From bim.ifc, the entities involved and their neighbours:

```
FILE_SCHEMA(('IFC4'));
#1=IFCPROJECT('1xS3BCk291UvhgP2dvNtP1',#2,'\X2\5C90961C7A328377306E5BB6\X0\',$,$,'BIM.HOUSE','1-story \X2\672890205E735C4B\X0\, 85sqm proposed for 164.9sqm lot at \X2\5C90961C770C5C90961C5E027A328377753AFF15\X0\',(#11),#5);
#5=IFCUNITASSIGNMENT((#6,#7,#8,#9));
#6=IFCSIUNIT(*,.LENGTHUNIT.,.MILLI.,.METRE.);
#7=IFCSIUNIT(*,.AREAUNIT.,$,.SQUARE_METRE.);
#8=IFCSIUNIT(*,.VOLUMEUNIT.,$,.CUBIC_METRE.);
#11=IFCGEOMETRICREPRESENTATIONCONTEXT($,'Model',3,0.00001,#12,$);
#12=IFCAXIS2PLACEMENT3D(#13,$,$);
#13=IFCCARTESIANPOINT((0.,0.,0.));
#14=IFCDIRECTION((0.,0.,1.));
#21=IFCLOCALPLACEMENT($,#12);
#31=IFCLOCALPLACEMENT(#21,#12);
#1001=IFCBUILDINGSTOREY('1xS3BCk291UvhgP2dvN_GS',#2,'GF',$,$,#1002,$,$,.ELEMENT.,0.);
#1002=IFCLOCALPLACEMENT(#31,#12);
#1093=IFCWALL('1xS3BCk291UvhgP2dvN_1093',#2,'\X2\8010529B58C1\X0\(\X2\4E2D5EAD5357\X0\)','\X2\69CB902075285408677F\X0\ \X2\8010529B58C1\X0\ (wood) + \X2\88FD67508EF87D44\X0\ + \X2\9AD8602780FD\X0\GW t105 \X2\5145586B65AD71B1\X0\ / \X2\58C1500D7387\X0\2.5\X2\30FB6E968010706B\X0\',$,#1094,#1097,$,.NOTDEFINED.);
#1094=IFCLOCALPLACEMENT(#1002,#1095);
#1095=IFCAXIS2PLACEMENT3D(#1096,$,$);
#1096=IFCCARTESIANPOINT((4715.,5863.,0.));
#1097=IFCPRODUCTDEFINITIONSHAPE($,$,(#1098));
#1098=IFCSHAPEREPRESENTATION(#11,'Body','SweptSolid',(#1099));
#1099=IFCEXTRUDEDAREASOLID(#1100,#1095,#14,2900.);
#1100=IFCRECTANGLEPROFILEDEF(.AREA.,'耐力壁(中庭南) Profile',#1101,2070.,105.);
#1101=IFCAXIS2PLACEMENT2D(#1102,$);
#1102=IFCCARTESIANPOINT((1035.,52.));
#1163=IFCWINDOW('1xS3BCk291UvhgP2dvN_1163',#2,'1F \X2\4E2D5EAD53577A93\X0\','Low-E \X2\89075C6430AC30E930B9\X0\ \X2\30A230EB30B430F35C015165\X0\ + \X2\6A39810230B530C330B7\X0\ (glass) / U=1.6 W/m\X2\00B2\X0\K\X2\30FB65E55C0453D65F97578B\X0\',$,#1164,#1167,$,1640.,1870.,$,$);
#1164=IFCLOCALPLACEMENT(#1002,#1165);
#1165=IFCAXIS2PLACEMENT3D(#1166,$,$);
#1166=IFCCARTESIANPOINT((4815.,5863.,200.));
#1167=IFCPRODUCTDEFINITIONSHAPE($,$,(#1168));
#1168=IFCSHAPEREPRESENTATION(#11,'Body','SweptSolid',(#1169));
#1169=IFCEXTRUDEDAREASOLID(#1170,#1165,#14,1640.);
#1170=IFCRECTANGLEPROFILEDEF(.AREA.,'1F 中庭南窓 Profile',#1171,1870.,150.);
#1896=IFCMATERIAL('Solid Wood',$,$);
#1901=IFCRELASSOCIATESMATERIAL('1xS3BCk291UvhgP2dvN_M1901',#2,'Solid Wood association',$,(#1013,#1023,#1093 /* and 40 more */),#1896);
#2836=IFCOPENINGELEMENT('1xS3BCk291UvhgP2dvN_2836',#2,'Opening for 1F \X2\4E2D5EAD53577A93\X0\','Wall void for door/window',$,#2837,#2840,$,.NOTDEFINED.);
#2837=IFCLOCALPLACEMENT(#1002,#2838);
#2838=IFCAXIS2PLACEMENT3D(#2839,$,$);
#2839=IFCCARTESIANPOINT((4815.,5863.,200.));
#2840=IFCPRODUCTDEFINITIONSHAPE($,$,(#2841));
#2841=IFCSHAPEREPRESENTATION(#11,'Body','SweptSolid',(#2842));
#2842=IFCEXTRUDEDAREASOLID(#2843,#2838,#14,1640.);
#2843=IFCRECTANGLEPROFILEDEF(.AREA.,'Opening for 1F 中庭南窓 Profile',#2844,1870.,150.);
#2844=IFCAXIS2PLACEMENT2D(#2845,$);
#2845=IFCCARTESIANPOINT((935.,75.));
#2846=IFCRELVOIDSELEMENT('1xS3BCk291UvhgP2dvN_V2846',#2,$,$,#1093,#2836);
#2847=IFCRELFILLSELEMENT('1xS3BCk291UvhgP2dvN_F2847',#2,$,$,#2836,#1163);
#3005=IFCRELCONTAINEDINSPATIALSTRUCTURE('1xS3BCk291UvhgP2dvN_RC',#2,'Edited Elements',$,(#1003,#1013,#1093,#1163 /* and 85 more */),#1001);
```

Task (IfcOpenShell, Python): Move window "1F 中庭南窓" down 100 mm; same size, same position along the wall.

```python
import numpy as np
import ifcopenshell
import ifcopenshell.api.geometry
import ifcopenshell.util.placement
import ifcopenshell.util.unit

model = ifcopenshell.open("bim.ifc")
unit_scale = ifcopenshell.util.unit.calculate_unit_scale(model)

window = model.by_guid("1xS3BCk291UvhgP2dvN_1163")
opening = window.FillsVoids[0].RelatingOpeningElement
dz = -100.0

shift = np.array([0.0, 0.0, dz])
# The window is not placed relative to its opening, so move both.
for product in (opening, window):
    matrix = ifcopenshell.util.placement.get_local_placement(product.ObjectPlacement)
    matrix[:3, 3] += shift
    ifcopenshell.api.geometry.edit_object_placement(model, product=product, matrix=matrix, is_si=False)

print(f"moved by {dz * unit_scale:+.3f} m")

model.write("bim_updated.ifc")
```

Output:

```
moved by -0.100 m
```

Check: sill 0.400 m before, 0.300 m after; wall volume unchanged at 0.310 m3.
